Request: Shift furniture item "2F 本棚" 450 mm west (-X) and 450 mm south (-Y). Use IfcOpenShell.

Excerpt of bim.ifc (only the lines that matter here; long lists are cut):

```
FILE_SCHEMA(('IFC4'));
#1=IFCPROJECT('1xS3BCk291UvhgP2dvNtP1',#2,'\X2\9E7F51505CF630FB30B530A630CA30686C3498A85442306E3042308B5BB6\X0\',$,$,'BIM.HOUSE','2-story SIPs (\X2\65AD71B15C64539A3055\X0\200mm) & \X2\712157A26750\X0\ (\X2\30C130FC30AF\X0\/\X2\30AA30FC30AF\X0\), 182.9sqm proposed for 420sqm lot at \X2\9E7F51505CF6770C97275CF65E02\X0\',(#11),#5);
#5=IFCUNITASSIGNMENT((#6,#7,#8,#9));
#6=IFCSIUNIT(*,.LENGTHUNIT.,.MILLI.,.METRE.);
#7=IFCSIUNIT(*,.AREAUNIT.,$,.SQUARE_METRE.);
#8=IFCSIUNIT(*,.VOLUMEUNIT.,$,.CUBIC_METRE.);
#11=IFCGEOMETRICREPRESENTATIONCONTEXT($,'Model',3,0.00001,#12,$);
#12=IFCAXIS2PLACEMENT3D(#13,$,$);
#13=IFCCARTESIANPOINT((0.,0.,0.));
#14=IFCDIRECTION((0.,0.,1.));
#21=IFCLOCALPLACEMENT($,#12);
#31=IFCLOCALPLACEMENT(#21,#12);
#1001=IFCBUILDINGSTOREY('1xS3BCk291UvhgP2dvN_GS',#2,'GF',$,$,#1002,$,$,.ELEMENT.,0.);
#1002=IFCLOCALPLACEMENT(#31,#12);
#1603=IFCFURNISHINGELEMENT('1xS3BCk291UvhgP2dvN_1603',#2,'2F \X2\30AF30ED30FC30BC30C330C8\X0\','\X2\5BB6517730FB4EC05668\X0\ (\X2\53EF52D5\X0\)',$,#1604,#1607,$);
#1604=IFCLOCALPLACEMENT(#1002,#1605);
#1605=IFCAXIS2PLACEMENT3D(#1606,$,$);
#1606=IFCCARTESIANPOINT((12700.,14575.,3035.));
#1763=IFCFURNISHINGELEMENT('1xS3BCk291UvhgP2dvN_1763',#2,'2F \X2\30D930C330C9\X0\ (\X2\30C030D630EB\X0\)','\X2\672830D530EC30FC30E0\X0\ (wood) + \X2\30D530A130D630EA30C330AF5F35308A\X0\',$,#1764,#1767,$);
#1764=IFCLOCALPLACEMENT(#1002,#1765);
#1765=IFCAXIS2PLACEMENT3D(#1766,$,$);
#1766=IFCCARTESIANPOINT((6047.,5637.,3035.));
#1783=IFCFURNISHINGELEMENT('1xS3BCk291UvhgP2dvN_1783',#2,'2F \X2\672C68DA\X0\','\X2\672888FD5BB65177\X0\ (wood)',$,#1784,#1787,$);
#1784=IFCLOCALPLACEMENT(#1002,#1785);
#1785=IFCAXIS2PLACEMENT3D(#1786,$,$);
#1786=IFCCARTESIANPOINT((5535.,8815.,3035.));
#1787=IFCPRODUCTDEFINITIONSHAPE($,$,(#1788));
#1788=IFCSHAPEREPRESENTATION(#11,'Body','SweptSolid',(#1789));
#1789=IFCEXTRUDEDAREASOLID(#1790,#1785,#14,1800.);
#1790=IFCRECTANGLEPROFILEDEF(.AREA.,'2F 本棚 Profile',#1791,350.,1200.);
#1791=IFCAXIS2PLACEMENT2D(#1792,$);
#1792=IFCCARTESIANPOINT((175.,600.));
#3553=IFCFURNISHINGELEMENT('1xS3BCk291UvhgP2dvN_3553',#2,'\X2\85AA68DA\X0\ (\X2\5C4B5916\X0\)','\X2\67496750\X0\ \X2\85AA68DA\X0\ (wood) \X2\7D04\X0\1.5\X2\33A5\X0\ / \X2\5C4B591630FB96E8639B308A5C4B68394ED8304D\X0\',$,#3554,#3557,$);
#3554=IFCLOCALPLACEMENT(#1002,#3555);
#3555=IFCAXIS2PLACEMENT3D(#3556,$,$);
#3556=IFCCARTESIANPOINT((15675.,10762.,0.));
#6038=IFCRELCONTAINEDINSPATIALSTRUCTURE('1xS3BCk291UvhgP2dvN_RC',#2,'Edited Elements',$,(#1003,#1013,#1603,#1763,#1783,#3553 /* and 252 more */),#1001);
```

```python
import ifcopenshell
import ifcopenshell.api.geometry
import ifcopenshell.util.placement
import ifcopenshell.util.unit

model = ifcopenshell.open("bim.ifc")
unit_scale = ifcopenshell.util.unit.calculate_unit_scale(model)

item = model.by_id(1783)
matrix = ifcopenshell.util.placement.get_local_placement(item.ObjectPlacement)
matrix[0, 3] -= 0.45 / unit_scale
matrix[1, 3] -= 0.45 / unit_scale
ifcopenshell.api.geometry.edit_object_placement(model, product=item, matrix=matrix, is_si=False)

print(ifcopenshell.util.placement.get_local_placement(item.ObjectPlacement).round(3) + 0.0)

model.write("bim_v2.ifc")
```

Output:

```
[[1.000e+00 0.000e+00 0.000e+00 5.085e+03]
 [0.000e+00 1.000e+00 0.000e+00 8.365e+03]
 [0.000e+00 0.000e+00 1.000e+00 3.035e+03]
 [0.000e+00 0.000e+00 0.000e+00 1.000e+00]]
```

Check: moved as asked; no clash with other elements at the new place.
